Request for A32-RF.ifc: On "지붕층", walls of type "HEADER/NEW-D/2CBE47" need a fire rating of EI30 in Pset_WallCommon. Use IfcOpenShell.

First a look at what the model holds.

```python
import ifcopenshell
import ifcopenshell.util.element

model = ifcopenshell.open("A32-RF.ifc")
print(model.schema)
storey = next(s for s in model.by_type("IfcBuildingStorey") if s.Name == "지붕층")
walls = [e for e in ifcopenshell.util.element.get_decomposition(storey) if e.is_a("IfcWall")]
seen = {}
for e in walls:
    element_type = ifcopenshell.util.element.get_type(e)
    key = (element_type.Name if element_type != e and element_type else None, ifcopenshell.util.element.get_pset(e, "Pset_WallCommon", "FireRating"))
    seen[key] = seen.get(key, 0) + 1
for (name, value), count in sorted(seen.items(), key=str):
    print(count, "x", name, "|", value)
```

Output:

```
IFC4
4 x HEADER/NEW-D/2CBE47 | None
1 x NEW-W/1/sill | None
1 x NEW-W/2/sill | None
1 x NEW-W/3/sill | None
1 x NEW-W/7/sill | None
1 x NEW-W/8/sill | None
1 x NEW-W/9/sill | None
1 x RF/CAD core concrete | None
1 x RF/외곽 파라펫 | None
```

```python
import ifcopenshell
import ifcopenshell.api.pset
import ifcopenshell.util.element

model = ifcopenshell.open("A32-RF.ifc")

storey = next(s for s in model.by_type("IfcBuildingStorey") if s.Name == "지붕층")
walls = [e for e in ifcopenshell.util.element.get_decomposition(storey) if e.is_a("IfcWall")]

count = 0
for e in walls:
    element_type = ifcopenshell.util.element.get_type(e)
    if element_type in (None, e) or element_type.Name != "HEADER/NEW-D/2CBE47":
        continue
    # add_pset returns the element's existing set when there is one.
    pset = ifcopenshell.api.pset.add_pset(model, product=e, name="Pset_WallCommon")
    ifcopenshell.api.pset.edit_pset(model, pset=pset, properties={"FireRating": "EI30"})
    count += 1

print(count, "walls updated")

model.write("A32-RF_updated.ifc")
```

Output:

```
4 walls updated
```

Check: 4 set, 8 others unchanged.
